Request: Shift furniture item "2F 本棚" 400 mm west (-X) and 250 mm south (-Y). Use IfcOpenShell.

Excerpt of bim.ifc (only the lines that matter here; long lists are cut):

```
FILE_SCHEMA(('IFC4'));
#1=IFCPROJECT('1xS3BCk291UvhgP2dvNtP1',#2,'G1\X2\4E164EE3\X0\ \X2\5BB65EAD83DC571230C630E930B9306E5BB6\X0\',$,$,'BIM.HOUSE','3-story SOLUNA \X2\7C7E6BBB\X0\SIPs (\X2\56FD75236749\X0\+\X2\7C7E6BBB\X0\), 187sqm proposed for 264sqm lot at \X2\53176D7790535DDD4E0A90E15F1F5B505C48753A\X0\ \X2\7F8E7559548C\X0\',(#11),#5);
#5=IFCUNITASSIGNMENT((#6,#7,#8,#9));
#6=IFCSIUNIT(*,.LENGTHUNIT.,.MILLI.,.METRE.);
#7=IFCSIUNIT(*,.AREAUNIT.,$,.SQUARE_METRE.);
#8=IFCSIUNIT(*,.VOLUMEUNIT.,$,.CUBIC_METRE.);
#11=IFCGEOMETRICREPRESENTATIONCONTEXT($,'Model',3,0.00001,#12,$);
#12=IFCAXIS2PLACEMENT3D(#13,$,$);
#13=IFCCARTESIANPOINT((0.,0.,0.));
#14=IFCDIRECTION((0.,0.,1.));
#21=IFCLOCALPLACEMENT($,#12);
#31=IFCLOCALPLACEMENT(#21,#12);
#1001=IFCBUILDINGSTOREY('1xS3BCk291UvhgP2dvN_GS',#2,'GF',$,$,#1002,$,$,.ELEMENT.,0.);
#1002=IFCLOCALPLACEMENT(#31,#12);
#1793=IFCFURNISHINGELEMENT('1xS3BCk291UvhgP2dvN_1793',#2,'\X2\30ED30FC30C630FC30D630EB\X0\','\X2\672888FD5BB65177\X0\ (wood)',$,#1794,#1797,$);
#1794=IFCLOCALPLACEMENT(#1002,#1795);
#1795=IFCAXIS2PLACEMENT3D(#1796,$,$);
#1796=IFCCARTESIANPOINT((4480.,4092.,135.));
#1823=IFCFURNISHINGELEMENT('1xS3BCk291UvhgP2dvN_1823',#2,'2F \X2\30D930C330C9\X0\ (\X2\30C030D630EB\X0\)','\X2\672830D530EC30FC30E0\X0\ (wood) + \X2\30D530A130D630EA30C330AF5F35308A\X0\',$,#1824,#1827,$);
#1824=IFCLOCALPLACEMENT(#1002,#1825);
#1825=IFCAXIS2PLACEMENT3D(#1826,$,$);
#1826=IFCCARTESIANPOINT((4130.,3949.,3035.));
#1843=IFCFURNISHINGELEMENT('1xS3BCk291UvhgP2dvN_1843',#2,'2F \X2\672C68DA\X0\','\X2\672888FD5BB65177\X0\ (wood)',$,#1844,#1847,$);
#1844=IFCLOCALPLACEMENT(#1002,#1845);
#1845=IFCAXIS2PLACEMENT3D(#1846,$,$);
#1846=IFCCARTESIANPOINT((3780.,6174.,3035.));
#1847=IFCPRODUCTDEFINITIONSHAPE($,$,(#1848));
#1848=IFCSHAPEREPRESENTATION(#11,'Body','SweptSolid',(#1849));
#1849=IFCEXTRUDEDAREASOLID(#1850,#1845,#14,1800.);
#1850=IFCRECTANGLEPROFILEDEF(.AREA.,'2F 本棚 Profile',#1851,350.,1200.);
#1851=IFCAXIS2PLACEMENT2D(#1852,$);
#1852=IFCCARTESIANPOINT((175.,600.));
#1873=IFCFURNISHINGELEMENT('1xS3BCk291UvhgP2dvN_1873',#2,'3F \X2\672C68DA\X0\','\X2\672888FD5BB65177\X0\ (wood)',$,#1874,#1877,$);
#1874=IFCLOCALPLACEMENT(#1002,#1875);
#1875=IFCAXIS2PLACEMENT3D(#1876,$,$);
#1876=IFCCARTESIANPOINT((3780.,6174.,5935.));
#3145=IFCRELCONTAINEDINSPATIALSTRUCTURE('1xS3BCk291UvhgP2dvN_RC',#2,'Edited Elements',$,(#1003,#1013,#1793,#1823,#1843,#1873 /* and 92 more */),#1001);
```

```python
import ifcopenshell
import ifcopenshell.api.geometry
import ifcopenshell.util.placement
import ifcopenshell.util.unit

model = ifcopenshell.open("bim.ifc")
unit_scale = ifcopenshell.util.unit.calculate_unit_scale(model)

item = model.by_guid("1xS3BCk291UvhgP2dvN_1843")
matrix = ifcopenshell.util.placement.get_local_placement(item.ObjectPlacement)
matrix[0, 3] -= 0.4 / unit_scale
matrix[1, 3] -= 0.25 / unit_scale
ifcopenshell.api.geometry.edit_object_placement(model, product=item, matrix=matrix, is_si=False)

print(ifcopenshell.util.placement.get_local_placement(item.ObjectPlacement).round(3) + 0.0)

model.write("bim_edited.ifc")
```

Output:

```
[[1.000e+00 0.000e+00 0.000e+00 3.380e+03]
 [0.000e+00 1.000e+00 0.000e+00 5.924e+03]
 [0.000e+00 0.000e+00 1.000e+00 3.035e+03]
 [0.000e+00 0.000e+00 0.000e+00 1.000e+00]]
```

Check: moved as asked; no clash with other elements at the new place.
